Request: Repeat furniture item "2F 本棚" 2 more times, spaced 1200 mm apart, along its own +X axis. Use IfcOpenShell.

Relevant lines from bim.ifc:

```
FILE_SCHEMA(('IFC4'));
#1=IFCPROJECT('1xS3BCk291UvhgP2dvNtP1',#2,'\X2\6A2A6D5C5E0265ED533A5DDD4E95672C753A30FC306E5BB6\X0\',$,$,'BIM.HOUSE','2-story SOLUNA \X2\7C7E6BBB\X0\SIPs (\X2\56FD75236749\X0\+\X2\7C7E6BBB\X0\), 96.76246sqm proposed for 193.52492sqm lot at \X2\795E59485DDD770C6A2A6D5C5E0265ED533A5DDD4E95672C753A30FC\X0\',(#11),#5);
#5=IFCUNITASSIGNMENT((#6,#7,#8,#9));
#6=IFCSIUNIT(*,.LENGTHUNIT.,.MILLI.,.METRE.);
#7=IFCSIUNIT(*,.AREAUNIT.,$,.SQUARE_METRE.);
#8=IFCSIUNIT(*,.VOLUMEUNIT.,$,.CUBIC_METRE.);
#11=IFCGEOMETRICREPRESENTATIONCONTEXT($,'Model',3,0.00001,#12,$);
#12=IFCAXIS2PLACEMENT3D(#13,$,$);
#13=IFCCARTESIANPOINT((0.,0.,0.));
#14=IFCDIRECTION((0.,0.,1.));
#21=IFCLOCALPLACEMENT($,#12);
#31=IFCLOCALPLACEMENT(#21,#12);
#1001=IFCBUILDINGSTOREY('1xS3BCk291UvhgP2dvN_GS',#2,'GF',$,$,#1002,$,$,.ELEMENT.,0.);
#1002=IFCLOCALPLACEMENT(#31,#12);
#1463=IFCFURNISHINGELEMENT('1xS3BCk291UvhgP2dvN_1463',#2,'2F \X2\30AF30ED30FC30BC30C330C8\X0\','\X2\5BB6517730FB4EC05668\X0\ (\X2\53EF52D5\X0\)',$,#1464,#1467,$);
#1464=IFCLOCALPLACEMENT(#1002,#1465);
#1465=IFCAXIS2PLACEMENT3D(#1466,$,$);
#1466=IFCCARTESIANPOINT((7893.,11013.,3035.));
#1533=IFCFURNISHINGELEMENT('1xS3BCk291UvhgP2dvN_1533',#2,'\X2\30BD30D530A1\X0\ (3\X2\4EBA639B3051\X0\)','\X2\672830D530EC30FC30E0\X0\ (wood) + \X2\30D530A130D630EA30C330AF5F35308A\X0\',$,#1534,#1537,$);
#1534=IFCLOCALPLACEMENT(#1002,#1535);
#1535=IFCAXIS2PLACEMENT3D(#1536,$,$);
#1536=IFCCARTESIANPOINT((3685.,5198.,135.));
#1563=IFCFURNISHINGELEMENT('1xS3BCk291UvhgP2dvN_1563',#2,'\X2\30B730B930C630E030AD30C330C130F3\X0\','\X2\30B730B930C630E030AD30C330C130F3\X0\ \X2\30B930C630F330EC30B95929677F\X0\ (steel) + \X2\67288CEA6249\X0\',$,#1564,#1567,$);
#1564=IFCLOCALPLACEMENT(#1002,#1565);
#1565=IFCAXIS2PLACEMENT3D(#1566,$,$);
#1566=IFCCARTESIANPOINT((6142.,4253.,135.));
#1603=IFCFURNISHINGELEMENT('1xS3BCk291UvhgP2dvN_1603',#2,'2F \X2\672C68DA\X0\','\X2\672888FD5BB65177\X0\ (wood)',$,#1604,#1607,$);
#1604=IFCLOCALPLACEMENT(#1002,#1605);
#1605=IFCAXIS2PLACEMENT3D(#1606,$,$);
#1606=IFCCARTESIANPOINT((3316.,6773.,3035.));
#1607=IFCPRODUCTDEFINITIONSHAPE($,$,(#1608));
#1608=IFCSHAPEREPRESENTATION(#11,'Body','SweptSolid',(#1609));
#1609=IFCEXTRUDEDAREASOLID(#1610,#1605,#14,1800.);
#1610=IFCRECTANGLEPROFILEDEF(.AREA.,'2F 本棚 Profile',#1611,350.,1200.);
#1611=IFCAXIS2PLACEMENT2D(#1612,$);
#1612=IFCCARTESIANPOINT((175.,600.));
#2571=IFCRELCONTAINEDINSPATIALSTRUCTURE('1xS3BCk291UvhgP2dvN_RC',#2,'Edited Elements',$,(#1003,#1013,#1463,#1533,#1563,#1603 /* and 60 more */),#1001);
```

```python
import ifcopenshell
import ifcopenshell.api.geometry
import ifcopenshell.api.root
import ifcopenshell.util.element
import ifcopenshell.util.placement

model = ifcopenshell.open("bim.ifc")


def reuse_history(source, copy):
    """copy_class also copies each property set's owner history, people and application; keep the originals."""
    for rel in copy.IsDefinedBy:
        if rel.is_a("IfcRelDefinesByProperties") and (history := rel.RelatingPropertyDefinition.OwnerHistory):
            rel.RelatingPropertyDefinition.OwnerHistory = source.OwnerHistory
            ifcopenshell.util.element.remove_deep2(model, history)


source = model.by_guid("1xS3BCk291UvhgP2dvN_1603")
base = ifcopenshell.util.placement.get_local_placement(source.ObjectPlacement)
step = base[:3, 0] * 1200.0

for i in range(1, 3):
    copy = ifcopenshell.api.root.copy_class(model, product=source)
    copy.Representation = ifcopenshell.util.element.copy_deep(
        model, source.Representation, exclude=["IfcGeometricRepresentationContext", "IfcRepresentationMap"]
    )
    reuse_history(source, copy)
    matrix = base.copy()
    matrix[:3, 3] += i * step
    print("added at", matrix[:3, 3].round(3) + 0.0)
    ifcopenshell.api.geometry.edit_object_placement(model, product=copy, matrix=matrix, is_si=False)

model.write("bim-out.ifc")
```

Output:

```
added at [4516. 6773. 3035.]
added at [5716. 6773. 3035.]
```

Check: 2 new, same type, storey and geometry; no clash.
